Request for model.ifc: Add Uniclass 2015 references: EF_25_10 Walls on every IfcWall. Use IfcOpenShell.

First a look at what the model holds.

```python
import ifcopenshell

model = ifcopenshell.open("model.ifc")
print(model.schema)
print("classifications:", [c.Name for c in model.by_type("IfcClassification")])
for ifc_class in ("IfcDoor", "IfcRoof", "IfcStair", "IfcWall", "IfcWindow"):
    print(ifc_class, len(model.by_type(ifc_class)))
```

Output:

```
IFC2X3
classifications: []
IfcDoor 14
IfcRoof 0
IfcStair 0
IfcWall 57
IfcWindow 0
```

```python
import ifcopenshell
import ifcopenshell.api.classification

model = ifcopenshell.open("model.ifc")

# IFC2X3 requires Source and Edition and has no link from the project to the system.
system = model.create_entity("IfcClassification", Source="NBS", Edition="2015", Name="Uniclass 2015")

codes = {
    "IfcWall": ("EF_25_10", "Walls"),
}
for ifc_class, (code, name) in codes.items():
    products = model.by_type(ifc_class)
    ifcopenshell.api.classification.add_reference(
        model, products=products, classification=system, identification=code, name=name
    )
    print(code, len(products))

model.write("model_edited.ifc")
```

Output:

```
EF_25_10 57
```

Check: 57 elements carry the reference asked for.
